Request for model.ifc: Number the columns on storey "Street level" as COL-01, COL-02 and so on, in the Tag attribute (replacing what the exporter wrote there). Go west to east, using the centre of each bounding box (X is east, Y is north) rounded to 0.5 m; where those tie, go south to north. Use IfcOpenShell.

First a look at what the model holds.

```python
import ifcopenshell
import ifcopenshell.util.element
import ifcopenshell.util.placement

model = ifcopenshell.open("model.ifc")
print(model.schema)
storey = next(s for s in model.by_type("IfcBuildingStorey") if s.Name == "Street level")
columns = [e for e in ifcopenshell.util.element.get_decomposition(storey) if e.is_a("IfcColumn")]
for e in sorted(columns, key=lambda e: e.id()):
    origin = ifcopenshell.util.placement.get_local_placement(e.ObjectPlacement)[:3, 3]
    print(e.id(), e.Tag, e.Name, origin.round(2) + 0.0, sep=" | ")
```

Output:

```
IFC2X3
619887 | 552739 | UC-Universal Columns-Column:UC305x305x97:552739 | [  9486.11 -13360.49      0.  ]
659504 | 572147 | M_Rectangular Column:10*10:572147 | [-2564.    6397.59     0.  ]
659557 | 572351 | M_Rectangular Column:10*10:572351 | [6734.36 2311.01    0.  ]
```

```python
import ifcopenshell
import ifcopenshell.geom
import ifcopenshell.util.element
import ifcopenshell.util.shape

model = ifcopenshell.open("model.ifc")
settings = ifcopenshell.geom.settings()
settings.set("use-world-coords", True)


def centre(element):
    shape = ifcopenshell.geom.create_shape(settings, element)
    return ifcopenshell.util.shape.get_bbox_centroid(shape.geometry)


storey = next(s for s in model.by_type("IfcBuildingStorey") if s.Name == "Street level")
columns = [e for e in ifcopenshell.util.element.get_decomposition(storey) if e.is_a("IfcColumn")]

# Insertion points can sit at a corner or the storey origin, so sort by the geometry (in metres).
centres = {e: centre(e) for e in columns}
columns.sort(key=lambda e: (round(centres[e][0] / 0.5), centres[e][1]))

for i, e in enumerate(columns, start=1):
    number = f"COL-{i:02d}"
    e.Tag = number
    print(e.id(), number)

model.write("model-out.ifc")
```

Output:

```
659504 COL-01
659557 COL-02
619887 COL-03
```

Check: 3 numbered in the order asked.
